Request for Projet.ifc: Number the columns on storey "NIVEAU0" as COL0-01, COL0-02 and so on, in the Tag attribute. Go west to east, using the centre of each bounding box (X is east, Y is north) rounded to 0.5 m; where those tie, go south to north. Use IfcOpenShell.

First a look at what the model holds.

```python
import ifcopenshell
import ifcopenshell.util.element
import ifcopenshell.util.placement

model = ifcopenshell.open("Projet.ifc")
print(model.schema)
storey = next(s for s in model.by_type("IfcBuildingStorey") if s.Name == "NIVEAU0")
columns = [e for e in ifcopenshell.util.element.get_decomposition(storey) if e.is_a("IfcColumn")]
for e in sorted(columns, key=lambda e: e.id()):
    origin = ifcopenshell.util.placement.get_local_placement(e.ObjectPlacement)[:3, 3]
    print(e.id(), e.Tag, e.Name, origin.round(2) + 0.0, sep=" | ")
```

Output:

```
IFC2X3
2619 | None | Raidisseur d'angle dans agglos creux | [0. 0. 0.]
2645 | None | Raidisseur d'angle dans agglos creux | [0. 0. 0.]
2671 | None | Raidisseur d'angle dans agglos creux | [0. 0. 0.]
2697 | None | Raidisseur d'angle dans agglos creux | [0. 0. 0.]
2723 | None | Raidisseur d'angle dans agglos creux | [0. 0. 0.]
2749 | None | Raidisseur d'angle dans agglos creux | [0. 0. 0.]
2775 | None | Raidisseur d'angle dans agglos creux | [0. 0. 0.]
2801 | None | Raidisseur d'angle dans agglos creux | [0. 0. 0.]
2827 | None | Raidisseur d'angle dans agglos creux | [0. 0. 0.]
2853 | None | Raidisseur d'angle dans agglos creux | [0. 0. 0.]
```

```python
import ifcopenshell
import ifcopenshell.geom
import ifcopenshell.util.element
import ifcopenshell.util.shape

model = ifcopenshell.open("Projet.ifc")
settings = ifcopenshell.geom.settings()
settings.set("use-world-coords", True)


def centre(element):
    shape = ifcopenshell.geom.create_shape(settings, element)
    return ifcopenshell.util.shape.get_bbox_centroid(shape.geometry)


storey = next(s for s in model.by_type("IfcBuildingStorey") if s.Name == "NIVEAU0")
columns = [e for e in ifcopenshell.util.element.get_decomposition(storey) if e.is_a("IfcColumn")]

# Insertion points can sit at a corner or the storey origin, so sort by the geometry (in metres).
centres = {e: centre(e) for e in columns}
columns.sort(key=lambda e: (round(centres[e][0] / 0.5), centres[e][1]))

for i, e in enumerate(columns, start=1):
    number = f"COL0-{i:02d}"
    e.Tag = number
    print(e.id(), number)

model.write("Projet_updated.ifc")
```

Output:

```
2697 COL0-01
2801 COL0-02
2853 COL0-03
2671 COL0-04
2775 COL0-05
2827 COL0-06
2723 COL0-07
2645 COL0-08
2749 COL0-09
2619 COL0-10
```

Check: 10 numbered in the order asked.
